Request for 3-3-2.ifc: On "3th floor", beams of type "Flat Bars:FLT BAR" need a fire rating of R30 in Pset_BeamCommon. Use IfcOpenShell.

First a look at what the model holds.

```python
import ifcopenshell
import ifcopenshell.util.element

model = ifcopenshell.open("3-3-2.ifc")
print(model.schema)
storey = next(s for s in model.by_type("IfcBuildingStorey") if s.Name == "3th floor")
beams = [e for e in ifcopenshell.util.element.get_decomposition(storey) if e.is_a("IfcBeam")]
seen = {}
for e in beams:
    element_type = ifcopenshell.util.element.get_type(e)
    key = (element_type.Name if element_type != e and element_type else None, ifcopenshell.util.element.get_pset(e, "Pset_BeamCommon", "FireRating"))
    seen[key] = seen.get(key, 0) + 1
for (name, value), count in sorted(seen.items(), key=str):
    print(count, "x", name, "|", value)
```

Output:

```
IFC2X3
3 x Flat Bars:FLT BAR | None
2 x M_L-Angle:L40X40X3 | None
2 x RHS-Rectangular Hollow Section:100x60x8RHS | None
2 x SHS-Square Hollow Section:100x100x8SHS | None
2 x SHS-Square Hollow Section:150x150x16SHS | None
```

```python
import ifcopenshell
import ifcopenshell.api.pset
import ifcopenshell.util.element

model = ifcopenshell.open("3-3-2.ifc")

storey = next(s for s in model.by_type("IfcBuildingStorey") if s.Name == "3th floor")
beams = [e for e in ifcopenshell.util.element.get_decomposition(storey) if e.is_a("IfcBeam")]

count = 0
for e in beams:
    element_type = ifcopenshell.util.element.get_type(e)
    if element_type in (None, e) or element_type.Name != "Flat Bars:FLT BAR":
        continue
    # add_pset returns the element's existing set when there is one.
    pset = ifcopenshell.api.pset.add_pset(model, product=e, name="Pset_BeamCommon")
    ifcopenshell.api.pset.edit_pset(model, pset=pset, properties={"FireRating": "R30"})
    count += 1

print(count, "beams updated")

model.write("3-3-2-out.ifc")
```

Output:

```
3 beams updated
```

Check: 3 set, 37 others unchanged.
